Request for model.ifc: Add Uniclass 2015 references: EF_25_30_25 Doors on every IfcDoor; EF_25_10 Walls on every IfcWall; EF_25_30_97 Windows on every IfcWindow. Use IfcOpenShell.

First a look at what the model holds.

```python
import ifcopenshell

model = ifcopenshell.open("model.ifc")
print(model.schema)
print("classifications:", [c.Name for c in model.by_type("IfcClassification")])
for ifc_class in ("IfcDoor", "IfcRoof", "IfcStair", "IfcWall", "IfcWindow"):
    print(ifc_class, len(model.by_type(ifc_class)))
```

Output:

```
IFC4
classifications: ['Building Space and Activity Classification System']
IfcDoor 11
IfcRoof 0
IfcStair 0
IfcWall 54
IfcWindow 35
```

```python
import ifcopenshell
import ifcopenshell.api.classification

model = ifcopenshell.open("model.ifc")

system = ifcopenshell.api.classification.add_classification(model, classification="Uniclass 2015")

codes = {
    "IfcDoor": ("EF_25_30_25", "Doors"),
    "IfcWall": ("EF_25_10", "Walls"),
    "IfcWindow": ("EF_25_30_97", "Windows"),
}
for ifc_class, (code, name) in codes.items():
    products = model.by_type(ifc_class)
    ifcopenshell.api.classification.add_reference(
        model, products=products, classification=system, identification=code, name=name
    )
    print(code, len(products))

model.write("model_updated.ifc")
```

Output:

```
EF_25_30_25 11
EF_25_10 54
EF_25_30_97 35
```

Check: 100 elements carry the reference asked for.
